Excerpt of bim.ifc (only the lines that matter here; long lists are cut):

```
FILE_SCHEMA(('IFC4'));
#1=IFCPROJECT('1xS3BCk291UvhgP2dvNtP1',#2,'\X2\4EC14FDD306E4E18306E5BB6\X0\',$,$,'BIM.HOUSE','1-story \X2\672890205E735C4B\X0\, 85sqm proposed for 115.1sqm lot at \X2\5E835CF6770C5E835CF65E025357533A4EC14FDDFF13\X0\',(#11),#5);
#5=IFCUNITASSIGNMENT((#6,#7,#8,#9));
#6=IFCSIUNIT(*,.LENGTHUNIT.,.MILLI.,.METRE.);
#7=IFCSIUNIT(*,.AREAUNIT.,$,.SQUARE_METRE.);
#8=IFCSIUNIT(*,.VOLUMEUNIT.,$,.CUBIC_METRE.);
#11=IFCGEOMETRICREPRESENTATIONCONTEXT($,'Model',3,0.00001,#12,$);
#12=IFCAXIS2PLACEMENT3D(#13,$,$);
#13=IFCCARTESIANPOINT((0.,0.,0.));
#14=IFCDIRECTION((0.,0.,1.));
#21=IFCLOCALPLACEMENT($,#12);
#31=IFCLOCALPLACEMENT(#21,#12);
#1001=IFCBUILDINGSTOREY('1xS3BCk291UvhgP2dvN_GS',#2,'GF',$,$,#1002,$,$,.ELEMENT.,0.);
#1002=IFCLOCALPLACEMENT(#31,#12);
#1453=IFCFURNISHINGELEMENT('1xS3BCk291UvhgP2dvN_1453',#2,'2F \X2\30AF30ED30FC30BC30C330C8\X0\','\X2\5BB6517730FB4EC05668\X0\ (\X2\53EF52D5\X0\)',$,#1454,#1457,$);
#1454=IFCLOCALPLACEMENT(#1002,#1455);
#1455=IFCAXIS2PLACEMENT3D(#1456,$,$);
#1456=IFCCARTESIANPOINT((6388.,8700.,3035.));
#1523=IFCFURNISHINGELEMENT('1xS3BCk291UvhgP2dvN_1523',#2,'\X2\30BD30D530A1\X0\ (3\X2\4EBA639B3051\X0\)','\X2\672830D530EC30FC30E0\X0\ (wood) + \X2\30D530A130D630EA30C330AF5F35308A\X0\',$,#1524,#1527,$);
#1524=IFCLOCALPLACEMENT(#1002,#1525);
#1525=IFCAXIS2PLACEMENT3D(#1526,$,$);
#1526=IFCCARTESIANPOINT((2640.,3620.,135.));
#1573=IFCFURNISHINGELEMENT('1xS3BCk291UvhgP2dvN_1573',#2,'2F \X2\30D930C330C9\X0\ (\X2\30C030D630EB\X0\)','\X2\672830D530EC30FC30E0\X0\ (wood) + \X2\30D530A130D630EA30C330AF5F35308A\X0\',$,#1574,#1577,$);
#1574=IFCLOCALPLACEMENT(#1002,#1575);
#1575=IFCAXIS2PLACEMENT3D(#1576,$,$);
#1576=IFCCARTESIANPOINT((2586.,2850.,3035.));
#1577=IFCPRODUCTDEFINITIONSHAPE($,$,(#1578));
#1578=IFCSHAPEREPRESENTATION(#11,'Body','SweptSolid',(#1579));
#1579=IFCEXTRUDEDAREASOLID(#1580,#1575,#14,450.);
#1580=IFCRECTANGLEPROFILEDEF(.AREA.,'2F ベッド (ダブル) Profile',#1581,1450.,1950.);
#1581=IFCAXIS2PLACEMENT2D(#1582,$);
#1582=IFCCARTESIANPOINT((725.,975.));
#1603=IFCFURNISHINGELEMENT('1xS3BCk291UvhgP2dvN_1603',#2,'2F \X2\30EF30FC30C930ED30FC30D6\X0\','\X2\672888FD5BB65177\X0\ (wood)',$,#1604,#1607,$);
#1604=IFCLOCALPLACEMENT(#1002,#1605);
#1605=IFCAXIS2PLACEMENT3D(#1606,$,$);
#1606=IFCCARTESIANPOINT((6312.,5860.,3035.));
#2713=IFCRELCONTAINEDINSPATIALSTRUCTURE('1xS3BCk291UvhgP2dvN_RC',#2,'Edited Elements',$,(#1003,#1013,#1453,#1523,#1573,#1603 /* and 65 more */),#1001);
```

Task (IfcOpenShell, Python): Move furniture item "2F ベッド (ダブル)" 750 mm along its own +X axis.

```python
import ifcopenshell
import ifcopenshell.api.geometry
import ifcopenshell.util.placement
import ifcopenshell.util.unit

model = ifcopenshell.open("bim.ifc")
unit_scale = ifcopenshell.util.unit.calculate_unit_scale(model)

item = model.by_guid("1xS3BCk291UvhgP2dvN_1573")
matrix = ifcopenshell.util.placement.get_local_placement(item.ObjectPlacement)
matrix[:3, 3] += matrix[:3, 0] * 0.75 / unit_scale
ifcopenshell.api.geometry.edit_object_placement(model, product=item, matrix=matrix, is_si=False)

print(ifcopenshell.util.placement.get_local_placement(item.ObjectPlacement).round(3) + 0.0)

model.write("bim_rev.ifc")
```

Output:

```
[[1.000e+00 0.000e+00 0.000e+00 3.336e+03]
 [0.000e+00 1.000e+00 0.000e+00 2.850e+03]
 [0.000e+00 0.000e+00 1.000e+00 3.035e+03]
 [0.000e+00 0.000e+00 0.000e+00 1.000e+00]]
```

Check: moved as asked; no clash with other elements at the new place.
